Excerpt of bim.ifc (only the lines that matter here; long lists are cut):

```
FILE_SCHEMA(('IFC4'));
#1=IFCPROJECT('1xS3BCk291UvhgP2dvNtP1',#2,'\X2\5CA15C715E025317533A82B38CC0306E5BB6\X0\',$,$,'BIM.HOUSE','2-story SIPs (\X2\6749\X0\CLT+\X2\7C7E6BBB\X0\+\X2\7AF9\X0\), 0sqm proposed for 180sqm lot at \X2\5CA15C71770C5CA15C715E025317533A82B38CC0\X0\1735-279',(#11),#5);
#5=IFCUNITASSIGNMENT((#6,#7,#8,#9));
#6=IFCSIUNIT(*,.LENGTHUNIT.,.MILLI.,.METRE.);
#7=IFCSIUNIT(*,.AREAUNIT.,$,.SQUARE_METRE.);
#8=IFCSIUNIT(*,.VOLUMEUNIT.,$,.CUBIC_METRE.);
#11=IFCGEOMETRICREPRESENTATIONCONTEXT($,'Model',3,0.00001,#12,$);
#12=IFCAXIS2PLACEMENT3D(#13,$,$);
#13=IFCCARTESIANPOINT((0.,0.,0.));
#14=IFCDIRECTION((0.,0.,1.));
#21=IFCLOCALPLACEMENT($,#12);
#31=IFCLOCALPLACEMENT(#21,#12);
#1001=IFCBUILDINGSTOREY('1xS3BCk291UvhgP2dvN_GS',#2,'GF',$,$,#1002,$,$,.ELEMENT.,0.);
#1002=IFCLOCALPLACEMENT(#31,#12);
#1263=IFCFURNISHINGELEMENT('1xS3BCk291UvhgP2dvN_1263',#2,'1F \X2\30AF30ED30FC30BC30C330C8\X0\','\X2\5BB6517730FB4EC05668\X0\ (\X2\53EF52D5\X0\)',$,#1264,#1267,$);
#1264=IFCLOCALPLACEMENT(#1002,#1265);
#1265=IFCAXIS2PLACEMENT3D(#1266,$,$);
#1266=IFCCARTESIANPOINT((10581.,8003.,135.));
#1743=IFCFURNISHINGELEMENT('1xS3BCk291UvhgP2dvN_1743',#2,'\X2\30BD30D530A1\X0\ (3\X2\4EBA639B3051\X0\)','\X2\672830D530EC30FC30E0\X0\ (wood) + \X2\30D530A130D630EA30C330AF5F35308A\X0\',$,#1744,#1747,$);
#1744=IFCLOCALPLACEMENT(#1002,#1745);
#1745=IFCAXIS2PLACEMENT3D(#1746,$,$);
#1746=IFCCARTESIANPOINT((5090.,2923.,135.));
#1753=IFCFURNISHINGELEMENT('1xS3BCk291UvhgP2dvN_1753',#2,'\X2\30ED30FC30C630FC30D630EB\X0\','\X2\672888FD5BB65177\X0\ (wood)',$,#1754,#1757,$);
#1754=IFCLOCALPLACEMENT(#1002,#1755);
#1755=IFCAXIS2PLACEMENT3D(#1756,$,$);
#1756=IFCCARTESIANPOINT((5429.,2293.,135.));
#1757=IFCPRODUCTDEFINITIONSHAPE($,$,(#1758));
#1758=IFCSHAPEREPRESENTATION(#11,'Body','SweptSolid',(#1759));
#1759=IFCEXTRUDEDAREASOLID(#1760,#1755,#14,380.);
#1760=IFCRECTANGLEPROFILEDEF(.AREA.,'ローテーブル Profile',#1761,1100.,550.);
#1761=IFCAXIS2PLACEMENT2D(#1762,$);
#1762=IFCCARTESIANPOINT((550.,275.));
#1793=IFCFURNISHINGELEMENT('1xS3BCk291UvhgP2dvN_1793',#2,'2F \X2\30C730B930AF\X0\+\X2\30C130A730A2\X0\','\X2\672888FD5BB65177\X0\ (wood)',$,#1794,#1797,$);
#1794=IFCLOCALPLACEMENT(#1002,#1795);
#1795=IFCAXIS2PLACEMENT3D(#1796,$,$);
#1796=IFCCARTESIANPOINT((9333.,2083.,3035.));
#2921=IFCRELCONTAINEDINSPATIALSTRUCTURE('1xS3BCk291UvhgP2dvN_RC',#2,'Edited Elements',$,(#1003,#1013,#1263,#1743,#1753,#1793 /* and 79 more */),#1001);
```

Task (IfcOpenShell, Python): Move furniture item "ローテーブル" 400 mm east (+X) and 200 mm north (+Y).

```python
import ifcopenshell
import ifcopenshell.api.geometry
import ifcopenshell.util.placement
import ifcopenshell.util.unit

model = ifcopenshell.open("bim.ifc")
unit_scale = ifcopenshell.util.unit.calculate_unit_scale(model)

item = model.by_guid("1xS3BCk291UvhgP2dvN_1753")
matrix = ifcopenshell.util.placement.get_local_placement(item.ObjectPlacement)
matrix[0, 3] += 0.4 / unit_scale
matrix[1, 3] += 0.2 / unit_scale
ifcopenshell.api.geometry.edit_object_placement(model, product=item, matrix=matrix, is_si=False)

print(ifcopenshell.util.placement.get_local_placement(item.ObjectPlacement).round(3) + 0.0)

model.write("bim-out.ifc")
```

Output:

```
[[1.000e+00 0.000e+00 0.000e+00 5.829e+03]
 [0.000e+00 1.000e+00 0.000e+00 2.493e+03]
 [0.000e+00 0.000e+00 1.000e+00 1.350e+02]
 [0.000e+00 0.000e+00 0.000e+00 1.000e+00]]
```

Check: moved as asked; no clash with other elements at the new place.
